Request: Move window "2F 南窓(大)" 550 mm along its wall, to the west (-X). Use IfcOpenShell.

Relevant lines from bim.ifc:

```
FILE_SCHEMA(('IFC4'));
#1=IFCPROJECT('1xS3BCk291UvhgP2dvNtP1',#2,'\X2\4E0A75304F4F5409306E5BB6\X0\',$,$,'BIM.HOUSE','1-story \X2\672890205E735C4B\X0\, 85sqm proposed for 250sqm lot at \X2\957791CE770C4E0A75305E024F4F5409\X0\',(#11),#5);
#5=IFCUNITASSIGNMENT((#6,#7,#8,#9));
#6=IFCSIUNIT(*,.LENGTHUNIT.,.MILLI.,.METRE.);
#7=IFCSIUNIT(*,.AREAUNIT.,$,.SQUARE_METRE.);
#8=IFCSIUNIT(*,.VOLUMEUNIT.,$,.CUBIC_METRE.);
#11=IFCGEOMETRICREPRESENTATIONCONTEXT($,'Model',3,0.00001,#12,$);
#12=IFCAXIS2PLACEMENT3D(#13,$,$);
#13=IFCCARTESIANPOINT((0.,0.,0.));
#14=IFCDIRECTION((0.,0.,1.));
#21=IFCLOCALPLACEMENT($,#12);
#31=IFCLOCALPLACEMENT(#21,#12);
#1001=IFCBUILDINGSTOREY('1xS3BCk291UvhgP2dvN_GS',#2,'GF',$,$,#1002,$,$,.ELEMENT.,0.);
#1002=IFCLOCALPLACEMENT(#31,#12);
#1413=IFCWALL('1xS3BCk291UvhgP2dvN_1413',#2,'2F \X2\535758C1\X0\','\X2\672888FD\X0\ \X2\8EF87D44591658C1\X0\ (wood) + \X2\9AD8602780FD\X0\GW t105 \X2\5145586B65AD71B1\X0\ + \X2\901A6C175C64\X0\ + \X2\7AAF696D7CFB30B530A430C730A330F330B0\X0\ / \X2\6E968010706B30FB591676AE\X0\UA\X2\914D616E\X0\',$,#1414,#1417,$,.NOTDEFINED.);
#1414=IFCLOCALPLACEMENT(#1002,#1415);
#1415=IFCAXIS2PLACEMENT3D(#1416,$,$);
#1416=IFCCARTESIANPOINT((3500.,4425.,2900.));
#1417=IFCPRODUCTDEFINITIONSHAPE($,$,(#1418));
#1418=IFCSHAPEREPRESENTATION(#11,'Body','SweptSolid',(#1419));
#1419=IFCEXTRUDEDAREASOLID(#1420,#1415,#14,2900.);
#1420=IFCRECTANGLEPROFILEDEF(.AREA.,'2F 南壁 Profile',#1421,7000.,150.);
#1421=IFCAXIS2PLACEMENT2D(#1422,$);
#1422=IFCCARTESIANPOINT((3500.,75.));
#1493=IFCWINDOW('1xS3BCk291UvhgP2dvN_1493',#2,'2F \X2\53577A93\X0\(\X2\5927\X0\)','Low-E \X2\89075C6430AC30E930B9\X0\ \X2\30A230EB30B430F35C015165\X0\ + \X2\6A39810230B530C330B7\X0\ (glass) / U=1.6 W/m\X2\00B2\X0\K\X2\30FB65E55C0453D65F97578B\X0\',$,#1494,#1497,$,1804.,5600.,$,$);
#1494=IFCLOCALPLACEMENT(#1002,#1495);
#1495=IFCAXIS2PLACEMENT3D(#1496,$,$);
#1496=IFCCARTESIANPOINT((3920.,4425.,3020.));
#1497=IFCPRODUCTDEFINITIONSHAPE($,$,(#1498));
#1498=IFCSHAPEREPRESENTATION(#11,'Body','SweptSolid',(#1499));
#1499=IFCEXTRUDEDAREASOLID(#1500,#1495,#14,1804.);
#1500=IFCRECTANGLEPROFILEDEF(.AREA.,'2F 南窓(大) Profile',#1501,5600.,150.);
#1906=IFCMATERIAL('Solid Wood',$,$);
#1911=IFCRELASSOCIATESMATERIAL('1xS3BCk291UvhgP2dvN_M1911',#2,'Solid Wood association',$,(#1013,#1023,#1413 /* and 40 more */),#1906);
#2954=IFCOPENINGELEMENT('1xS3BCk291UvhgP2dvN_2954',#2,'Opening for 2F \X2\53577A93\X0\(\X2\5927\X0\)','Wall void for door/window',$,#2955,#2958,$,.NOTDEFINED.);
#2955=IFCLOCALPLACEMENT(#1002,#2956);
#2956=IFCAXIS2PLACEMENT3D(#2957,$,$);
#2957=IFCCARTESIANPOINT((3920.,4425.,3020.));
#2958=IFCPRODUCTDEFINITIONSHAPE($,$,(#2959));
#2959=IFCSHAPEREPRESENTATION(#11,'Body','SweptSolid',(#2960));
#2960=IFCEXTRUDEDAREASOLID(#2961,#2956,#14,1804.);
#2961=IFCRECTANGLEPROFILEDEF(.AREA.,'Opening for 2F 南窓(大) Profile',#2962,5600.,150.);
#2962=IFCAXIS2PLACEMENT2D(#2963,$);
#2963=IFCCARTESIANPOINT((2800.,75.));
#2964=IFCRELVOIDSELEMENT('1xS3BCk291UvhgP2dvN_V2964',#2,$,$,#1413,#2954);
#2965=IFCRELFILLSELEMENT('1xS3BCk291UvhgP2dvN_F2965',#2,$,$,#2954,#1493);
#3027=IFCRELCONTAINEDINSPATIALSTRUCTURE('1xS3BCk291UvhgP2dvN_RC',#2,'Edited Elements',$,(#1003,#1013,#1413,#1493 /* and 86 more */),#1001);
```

```python
import ifcopenshell
import ifcopenshell.api.geometry
import ifcopenshell.util.placement
import ifcopenshell.util.unit

model = ifcopenshell.open("bim.ifc")
unit_scale = ifcopenshell.util.unit.calculate_unit_scale(model)

window = model.by_guid("1xS3BCk291UvhgP2dvN_1493")
opening = window.FillsVoids[0].RelatingOpeningElement
wall = opening.VoidsElements[0].RelatingBuildingElement

wall_matrix = ifcopenshell.util.placement.get_local_placement(wall.ObjectPlacement)
shift = wall_matrix[:3, 0] * -0.55 / unit_scale
before = ifcopenshell.util.placement.get_local_placement(window.ObjectPlacement)[:3, 3].copy()

# The window is not placed relative to its opening, so move both.
for product in (opening, window):
    matrix = ifcopenshell.util.placement.get_local_placement(product.ObjectPlacement)
    matrix[:3, 3] += shift
    ifcopenshell.api.geometry.edit_object_placement(model, product=product, matrix=matrix, is_si=False)

after = ifcopenshell.util.placement.get_local_placement(window.ObjectPlacement)[:3, 3]
print("window moved by", (after - before).round(3) + 0.0)

model.write("bim-out.ifc")
```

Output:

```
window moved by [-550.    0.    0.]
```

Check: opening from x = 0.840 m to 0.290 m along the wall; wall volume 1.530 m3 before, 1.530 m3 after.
